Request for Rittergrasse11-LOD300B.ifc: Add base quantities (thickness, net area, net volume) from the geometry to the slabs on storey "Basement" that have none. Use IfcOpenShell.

First a look at what the model holds.

```python
import ifcopenshell
import ifcopenshell.util.element
import ifcopenshell.util.unit

model = ifcopenshell.open("Rittergrasse11-LOD300B.ifc")
print(model.schema)
for unit_type in ("LENGTHUNIT", "AREAUNIT", "VOLUMEUNIT"):
    print(unit_type, ifcopenshell.util.unit.calculate_unit_scale(model, unit_type))
storey = next(s for s in model.by_type("IfcBuildingStorey") if s.Name == "Basement")
slabs = [e for e in ifcopenshell.util.element.get_decomposition(storey) if e.is_a("IfcSlab")]
for e in sorted(slabs, key=lambda e: e.id()):
    print(e.id(), e.is_a(), e.Name, list(ifcopenshell.util.element.get_psets(e, qtos_only=True)), sep=" | ")
```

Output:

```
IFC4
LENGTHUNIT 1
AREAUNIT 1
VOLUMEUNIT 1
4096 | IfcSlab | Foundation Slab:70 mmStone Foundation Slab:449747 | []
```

```python
import ifcopenshell
import ifcopenshell.api.pset
import ifcopenshell.geom
import ifcopenshell.util.element
import ifcopenshell.util.shape
import ifcopenshell.util.unit

model = ifcopenshell.open("Rittergrasse11-LOD300B.ifc")
unit_scale = ifcopenshell.util.unit.calculate_unit_scale(model)
area_scale = ifcopenshell.util.unit.calculate_unit_scale(model, "AREAUNIT")
volume_scale = ifcopenshell.util.unit.calculate_unit_scale(model, "VOLUMEUNIT")
settings = ifcopenshell.geom.settings()

storey = next(s for s in model.by_type("IfcBuildingStorey") if s.Name == "Basement")
slabs = [e for e in ifcopenshell.util.element.get_decomposition(storey) if e.is_a("IfcSlab")]

for e in sorted(slabs, key=lambda e: e.id()):
    if ifcopenshell.util.element.get_psets(e, qtos_only=True, should_inherit=False):
        continue
    # Geometry comes back in metres, in the element's own axes.
    shape = ifcopenshell.geom.create_shape(settings, e)
    values = {
        "Width": ifcopenshell.util.shape.get_z(shape.geometry) / unit_scale,
        "NetArea": ifcopenshell.util.shape.get_footprint_area(shape.geometry) / area_scale,
        "NetVolume": ifcopenshell.util.shape.get_volume(shape.geometry) / volume_scale,
    }
    qto = ifcopenshell.api.pset.add_qto(model, product=e, name="Qto_SlabBaseQuantities")
    ifcopenshell.api.pset.edit_qto(model, qto=qto, properties=values)
    print(e.id(), {k: round(v, 3) for k, v in values.items()})

model.write("Rittergrasse11-LOD300B_edited.ifc")
```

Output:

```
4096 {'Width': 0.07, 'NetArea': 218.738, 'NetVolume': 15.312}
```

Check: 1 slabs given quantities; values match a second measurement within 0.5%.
